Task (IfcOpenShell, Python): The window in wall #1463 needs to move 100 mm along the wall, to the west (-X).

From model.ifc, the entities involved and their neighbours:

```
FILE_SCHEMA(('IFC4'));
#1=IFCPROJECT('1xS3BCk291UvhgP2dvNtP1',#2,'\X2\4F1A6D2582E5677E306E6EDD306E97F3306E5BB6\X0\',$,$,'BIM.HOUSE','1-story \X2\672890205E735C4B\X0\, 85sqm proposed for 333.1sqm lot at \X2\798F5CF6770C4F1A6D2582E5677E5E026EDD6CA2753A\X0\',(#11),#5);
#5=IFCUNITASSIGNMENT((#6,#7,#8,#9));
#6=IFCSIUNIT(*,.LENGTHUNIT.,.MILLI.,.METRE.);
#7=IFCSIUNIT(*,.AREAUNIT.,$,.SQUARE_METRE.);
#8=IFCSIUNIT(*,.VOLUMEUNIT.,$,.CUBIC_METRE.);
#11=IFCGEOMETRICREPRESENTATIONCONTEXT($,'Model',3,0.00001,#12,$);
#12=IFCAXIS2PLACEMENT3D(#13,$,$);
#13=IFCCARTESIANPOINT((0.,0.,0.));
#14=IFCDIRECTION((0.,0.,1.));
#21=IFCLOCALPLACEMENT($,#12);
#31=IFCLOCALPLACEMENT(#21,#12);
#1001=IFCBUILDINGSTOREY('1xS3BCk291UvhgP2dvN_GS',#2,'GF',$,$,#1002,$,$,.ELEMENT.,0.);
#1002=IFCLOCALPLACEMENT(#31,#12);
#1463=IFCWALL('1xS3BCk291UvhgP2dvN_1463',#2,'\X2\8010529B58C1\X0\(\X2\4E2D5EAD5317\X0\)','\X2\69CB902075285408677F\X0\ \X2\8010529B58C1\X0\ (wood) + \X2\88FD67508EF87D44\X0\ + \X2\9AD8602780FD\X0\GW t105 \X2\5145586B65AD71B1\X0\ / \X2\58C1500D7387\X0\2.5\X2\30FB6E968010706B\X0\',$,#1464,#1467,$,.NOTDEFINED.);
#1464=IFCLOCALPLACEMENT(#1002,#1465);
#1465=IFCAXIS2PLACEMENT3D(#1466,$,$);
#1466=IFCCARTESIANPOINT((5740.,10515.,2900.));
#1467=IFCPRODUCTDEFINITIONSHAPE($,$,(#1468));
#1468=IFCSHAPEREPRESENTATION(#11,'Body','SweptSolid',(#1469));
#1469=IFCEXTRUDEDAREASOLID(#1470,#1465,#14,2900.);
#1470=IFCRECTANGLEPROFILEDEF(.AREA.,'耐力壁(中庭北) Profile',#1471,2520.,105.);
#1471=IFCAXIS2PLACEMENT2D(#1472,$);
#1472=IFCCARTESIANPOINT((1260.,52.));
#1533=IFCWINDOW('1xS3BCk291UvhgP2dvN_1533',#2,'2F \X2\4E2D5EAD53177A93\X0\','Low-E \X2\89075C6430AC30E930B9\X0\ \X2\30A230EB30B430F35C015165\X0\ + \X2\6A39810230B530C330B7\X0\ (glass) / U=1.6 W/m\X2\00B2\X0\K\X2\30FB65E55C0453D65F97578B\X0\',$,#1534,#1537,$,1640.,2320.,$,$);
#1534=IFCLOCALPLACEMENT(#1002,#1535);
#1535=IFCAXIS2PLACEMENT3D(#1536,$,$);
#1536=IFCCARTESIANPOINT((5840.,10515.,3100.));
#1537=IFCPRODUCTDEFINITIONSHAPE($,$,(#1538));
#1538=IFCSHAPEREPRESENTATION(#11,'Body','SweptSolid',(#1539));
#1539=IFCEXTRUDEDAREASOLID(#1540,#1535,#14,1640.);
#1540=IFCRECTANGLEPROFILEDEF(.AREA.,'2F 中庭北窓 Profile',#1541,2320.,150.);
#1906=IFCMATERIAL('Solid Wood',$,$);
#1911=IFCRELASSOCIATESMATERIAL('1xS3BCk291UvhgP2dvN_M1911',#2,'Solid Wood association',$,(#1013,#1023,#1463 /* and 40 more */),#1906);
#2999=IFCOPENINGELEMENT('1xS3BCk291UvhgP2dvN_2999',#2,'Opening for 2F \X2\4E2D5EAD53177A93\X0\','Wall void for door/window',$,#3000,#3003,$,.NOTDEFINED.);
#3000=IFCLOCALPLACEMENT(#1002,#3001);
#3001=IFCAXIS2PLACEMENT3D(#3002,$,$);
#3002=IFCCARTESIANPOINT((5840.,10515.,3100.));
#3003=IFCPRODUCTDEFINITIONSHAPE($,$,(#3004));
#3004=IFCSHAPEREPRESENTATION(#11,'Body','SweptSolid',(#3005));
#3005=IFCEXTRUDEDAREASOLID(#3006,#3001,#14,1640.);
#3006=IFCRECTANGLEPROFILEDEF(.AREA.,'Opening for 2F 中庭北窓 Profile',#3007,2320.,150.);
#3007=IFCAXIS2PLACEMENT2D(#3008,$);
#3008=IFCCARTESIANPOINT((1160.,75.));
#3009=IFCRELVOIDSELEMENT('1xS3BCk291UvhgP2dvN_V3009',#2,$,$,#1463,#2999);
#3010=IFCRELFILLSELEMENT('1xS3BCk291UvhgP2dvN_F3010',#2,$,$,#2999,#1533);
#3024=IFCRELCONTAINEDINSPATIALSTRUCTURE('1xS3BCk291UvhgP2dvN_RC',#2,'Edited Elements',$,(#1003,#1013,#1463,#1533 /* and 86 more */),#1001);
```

```python
import ifcopenshell
import ifcopenshell.api.geometry
import ifcopenshell.util.placement

model = ifcopenshell.open("model.ifc")

window = model.by_guid("1xS3BCk291UvhgP2dvN_1533")
opening = window.FillsVoids[0].RelatingOpeningElement
wall = opening.VoidsElements[0].RelatingBuildingElement

wall_matrix = ifcopenshell.util.placement.get_local_placement(wall.ObjectPlacement)
shift = wall_matrix[:3, 0] * -100.0
before = ifcopenshell.util.placement.get_local_placement(window.ObjectPlacement)[:3, 3].copy()

# The window is not placed relative to its opening, so move both.
for product in (opening, window):
    matrix = ifcopenshell.util.placement.get_local_placement(product.ObjectPlacement)
    matrix[:3, 3] += shift
    ifcopenshell.api.geometry.edit_object_placement(model, product=product, matrix=matrix, is_si=False)

after = ifcopenshell.util.placement.get_local_placement(window.ObjectPlacement)[:3, 3]
print("window moved by", (after - before).round(3) + 0.0)

model.write("model_v2.ifc")
```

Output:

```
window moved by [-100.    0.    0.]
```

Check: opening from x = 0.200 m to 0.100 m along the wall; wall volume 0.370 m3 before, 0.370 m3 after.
